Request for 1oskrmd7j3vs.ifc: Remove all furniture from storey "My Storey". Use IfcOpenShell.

First a look at what the model holds.

```python
import ifcopenshell
import ifcopenshell.util.element

model = ifcopenshell.open("1oskrmd7j3vs.ifc")
print(model.schema)
storey = next(s for s in model.by_type("IfcBuildingStorey") if s.Name == "My Storey")
furniture = [e for e in ifcopenshell.util.element.get_decomposition(storey) if e.is_a("IfcFurnishingElement")]
seen = {}
for e in furniture:
    element_type = ifcopenshell.util.element.get_type(e)
    name = element_type.Name if element_type not in (None, e) else None
    seen[name] = seen.get(name, 0) + 1
for name, count in sorted(seen.items(), key=str):
    print(count, "x", name)
```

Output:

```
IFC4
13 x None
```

```python
import ifcopenshell
import ifcopenshell.api.root
import ifcopenshell.util.element

model = ifcopenshell.open("1oskrmd7j3vs.ifc")

storey = next(s for s in model.by_type("IfcBuildingStorey") if s.Name == "My Storey")
furniture = [e for e in ifcopenshell.util.element.get_decomposition(storey) if e.is_a("IfcFurnishingElement")]

for e in furniture:
    ifcopenshell.api.root.remove_product(model, product=e)
print(len(furniture), "removed")

model.write("1oskrmd7j3vs-out.ifc")
```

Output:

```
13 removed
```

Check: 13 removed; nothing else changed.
